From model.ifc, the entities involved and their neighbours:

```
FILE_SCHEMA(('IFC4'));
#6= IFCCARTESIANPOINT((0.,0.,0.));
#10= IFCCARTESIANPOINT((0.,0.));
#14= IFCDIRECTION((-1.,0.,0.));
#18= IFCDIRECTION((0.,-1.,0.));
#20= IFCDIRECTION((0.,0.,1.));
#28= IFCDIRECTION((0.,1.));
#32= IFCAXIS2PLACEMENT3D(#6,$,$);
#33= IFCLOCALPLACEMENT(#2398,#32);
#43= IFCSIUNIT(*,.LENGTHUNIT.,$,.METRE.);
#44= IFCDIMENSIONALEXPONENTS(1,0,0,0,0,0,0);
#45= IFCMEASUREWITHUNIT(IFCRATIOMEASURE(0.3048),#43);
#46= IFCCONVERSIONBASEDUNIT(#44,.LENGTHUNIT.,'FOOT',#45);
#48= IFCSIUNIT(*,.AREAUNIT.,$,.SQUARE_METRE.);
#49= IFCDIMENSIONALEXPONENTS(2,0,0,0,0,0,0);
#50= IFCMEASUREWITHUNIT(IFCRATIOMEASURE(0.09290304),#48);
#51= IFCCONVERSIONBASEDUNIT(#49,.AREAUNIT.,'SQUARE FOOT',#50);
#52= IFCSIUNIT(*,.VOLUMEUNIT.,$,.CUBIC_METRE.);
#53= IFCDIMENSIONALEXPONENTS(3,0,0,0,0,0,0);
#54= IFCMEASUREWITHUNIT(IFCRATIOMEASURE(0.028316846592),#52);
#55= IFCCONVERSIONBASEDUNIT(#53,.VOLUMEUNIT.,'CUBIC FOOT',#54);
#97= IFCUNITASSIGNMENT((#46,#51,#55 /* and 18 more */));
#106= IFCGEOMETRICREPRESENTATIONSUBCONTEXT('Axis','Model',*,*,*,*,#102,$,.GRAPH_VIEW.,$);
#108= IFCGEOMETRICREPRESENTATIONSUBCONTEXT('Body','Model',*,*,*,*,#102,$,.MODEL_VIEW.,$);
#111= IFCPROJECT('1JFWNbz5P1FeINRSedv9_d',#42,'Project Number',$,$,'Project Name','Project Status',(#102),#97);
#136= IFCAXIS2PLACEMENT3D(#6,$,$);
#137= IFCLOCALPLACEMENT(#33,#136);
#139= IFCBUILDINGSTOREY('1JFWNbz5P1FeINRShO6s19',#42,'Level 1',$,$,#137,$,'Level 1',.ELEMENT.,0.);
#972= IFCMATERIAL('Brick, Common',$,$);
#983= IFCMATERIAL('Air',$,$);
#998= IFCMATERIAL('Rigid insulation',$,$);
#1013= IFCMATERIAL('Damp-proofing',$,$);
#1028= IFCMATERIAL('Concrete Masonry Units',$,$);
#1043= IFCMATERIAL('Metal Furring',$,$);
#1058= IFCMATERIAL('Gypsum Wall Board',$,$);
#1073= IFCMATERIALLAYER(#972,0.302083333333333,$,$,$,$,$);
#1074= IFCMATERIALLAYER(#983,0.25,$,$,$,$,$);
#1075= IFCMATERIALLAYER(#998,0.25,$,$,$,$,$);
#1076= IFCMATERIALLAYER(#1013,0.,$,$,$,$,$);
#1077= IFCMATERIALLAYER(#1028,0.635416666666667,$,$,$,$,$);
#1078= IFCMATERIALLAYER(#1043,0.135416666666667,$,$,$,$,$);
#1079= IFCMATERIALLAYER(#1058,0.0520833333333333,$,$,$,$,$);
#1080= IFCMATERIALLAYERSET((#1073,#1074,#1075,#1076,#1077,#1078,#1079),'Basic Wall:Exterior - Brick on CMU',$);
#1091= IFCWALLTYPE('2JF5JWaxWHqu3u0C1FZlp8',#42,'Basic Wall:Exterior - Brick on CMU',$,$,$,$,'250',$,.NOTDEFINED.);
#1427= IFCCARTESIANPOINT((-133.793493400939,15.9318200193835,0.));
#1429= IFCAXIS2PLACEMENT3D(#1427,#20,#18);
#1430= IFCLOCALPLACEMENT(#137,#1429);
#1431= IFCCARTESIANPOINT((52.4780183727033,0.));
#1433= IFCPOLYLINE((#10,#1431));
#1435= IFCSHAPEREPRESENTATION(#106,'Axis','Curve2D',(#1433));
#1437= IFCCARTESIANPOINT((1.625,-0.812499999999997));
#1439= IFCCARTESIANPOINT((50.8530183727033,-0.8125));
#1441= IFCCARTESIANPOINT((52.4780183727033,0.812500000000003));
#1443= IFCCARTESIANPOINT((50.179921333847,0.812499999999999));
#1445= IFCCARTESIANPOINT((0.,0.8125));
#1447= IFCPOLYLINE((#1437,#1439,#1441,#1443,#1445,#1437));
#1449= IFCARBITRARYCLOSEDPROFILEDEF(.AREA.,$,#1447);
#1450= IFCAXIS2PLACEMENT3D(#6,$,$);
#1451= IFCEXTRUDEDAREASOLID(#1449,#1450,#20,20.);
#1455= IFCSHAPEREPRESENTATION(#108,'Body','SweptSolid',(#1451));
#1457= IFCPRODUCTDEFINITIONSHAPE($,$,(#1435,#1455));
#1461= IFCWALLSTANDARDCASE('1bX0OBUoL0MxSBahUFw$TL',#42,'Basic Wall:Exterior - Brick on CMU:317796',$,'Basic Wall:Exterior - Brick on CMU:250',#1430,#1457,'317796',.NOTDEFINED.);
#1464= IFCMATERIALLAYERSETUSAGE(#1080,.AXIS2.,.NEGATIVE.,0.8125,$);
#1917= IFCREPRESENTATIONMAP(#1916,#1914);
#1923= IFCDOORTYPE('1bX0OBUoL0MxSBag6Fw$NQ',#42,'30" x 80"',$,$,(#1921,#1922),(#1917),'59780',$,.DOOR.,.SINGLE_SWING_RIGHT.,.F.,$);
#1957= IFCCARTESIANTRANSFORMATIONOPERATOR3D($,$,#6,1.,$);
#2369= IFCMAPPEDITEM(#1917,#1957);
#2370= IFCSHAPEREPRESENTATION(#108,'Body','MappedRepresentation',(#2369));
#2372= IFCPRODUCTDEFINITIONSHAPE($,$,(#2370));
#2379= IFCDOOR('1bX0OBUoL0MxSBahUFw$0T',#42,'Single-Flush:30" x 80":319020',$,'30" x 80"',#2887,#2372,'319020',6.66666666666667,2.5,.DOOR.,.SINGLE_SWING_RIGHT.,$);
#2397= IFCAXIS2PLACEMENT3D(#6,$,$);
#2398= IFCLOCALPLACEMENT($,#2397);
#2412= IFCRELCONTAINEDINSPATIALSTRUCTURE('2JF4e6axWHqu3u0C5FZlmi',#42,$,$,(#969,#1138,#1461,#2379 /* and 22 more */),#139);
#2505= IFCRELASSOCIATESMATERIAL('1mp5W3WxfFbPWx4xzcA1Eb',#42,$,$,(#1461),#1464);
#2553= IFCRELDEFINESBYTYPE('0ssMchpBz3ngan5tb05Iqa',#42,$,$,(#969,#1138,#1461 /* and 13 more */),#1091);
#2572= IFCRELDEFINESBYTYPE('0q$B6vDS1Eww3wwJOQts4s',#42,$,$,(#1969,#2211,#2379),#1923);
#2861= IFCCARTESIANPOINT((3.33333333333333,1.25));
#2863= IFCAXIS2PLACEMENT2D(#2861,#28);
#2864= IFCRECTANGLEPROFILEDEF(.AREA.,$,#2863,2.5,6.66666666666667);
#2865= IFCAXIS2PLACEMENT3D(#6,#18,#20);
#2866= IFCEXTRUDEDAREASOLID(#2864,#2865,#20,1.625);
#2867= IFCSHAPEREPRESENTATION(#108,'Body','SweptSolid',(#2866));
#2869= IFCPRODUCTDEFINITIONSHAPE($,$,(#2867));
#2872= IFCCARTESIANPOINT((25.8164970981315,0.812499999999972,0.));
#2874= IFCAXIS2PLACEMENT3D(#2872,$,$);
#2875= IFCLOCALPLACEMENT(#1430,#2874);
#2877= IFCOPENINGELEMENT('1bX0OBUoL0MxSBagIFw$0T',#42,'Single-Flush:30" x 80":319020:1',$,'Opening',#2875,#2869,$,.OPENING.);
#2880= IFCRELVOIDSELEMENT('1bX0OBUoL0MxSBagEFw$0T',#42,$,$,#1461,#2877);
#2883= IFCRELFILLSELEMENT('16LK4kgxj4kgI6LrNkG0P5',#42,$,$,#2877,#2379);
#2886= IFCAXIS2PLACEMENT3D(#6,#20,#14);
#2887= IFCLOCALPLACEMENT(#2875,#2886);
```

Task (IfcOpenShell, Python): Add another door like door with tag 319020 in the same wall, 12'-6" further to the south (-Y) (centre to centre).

```python
import ifcopenshell
import ifcopenshell.api.feature
import ifcopenshell.api.geometry
import ifcopenshell.api.root
import ifcopenshell.geom
import ifcopenshell.util.element
import ifcopenshell.util.placement
import ifcopenshell.util.shape
import ifcopenshell.util.unit

model = ifcopenshell.open("model.ifc")
unit_scale = ifcopenshell.util.unit.calculate_unit_scale(model)
settings = ifcopenshell.geom.settings()


def volume(element):
    """Net volume in cubic metres, openings subtracted."""
    shape = ifcopenshell.geom.create_shape(settings, element)
    return ifcopenshell.util.shape.get_volume(shape.geometry)


def reuse_history(source, copy):
    """copy_class also copies each property set's owner history, people and application; keep the originals."""
    for rel in copy.IsDefinedBy:
        if rel.is_a("IfcRelDefinesByProperties") and (history := rel.RelatingPropertyDefinition.OwnerHistory):
            rel.RelatingPropertyDefinition.OwnerHistory = source.OwnerHistory
            ifcopenshell.util.element.remove_deep2(model, history)


door = model.by_guid("1bX0OBUoL0MxSBahUFw$0T")
opening = door.FillsVoids[0].RelatingOpeningElement
wall = opening.VoidsElements[0].RelatingBuildingElement
before = volume(wall)
shift = ifcopenshell.util.placement.get_local_placement(wall.ObjectPlacement)[:3, 0] * 150 * 0.0254 / unit_scale

# copy_class copies the void relationship, type, container and properties, but no geometry.
new_opening = ifcopenshell.api.root.copy_class(model, product=opening)
new_opening.Representation = ifcopenshell.util.element.copy_deep(
    model, opening.Representation, exclude=["IfcGeometricRepresentationContext", "IfcRepresentationMap"]
)
new_opening.Name = 'Single-Flush:30" x 80"'
new_door = ifcopenshell.api.root.copy_class(model, product=door)
new_door.Representation = ifcopenshell.util.element.copy_deep(
    model, door.Representation, exclude=["IfcGeometricRepresentationContext", "IfcRepresentationMap"]
)
new_door.Name = 'Single-Flush:30" x 80"'
new_door.Tag = None
reuse_history(door, new_door)
ifcopenshell.api.feature.add_filling(model, opening=new_opening, element=new_door)

for old, new in ((opening, new_opening), (door, new_door)):
    matrix = ifcopenshell.util.placement.get_local_placement(old.ObjectPlacement)
    matrix[:3, 3] += shift
    ifcopenshell.api.geometry.edit_object_placement(model, product=new, matrix=matrix, is_si=False)

after = volume(wall)

print(f"wall volume {before:.3f} -> {after:.3f} m3")

model.write("model_rev.ifc")
```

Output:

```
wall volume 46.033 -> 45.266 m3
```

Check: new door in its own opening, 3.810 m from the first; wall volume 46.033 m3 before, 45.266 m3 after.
